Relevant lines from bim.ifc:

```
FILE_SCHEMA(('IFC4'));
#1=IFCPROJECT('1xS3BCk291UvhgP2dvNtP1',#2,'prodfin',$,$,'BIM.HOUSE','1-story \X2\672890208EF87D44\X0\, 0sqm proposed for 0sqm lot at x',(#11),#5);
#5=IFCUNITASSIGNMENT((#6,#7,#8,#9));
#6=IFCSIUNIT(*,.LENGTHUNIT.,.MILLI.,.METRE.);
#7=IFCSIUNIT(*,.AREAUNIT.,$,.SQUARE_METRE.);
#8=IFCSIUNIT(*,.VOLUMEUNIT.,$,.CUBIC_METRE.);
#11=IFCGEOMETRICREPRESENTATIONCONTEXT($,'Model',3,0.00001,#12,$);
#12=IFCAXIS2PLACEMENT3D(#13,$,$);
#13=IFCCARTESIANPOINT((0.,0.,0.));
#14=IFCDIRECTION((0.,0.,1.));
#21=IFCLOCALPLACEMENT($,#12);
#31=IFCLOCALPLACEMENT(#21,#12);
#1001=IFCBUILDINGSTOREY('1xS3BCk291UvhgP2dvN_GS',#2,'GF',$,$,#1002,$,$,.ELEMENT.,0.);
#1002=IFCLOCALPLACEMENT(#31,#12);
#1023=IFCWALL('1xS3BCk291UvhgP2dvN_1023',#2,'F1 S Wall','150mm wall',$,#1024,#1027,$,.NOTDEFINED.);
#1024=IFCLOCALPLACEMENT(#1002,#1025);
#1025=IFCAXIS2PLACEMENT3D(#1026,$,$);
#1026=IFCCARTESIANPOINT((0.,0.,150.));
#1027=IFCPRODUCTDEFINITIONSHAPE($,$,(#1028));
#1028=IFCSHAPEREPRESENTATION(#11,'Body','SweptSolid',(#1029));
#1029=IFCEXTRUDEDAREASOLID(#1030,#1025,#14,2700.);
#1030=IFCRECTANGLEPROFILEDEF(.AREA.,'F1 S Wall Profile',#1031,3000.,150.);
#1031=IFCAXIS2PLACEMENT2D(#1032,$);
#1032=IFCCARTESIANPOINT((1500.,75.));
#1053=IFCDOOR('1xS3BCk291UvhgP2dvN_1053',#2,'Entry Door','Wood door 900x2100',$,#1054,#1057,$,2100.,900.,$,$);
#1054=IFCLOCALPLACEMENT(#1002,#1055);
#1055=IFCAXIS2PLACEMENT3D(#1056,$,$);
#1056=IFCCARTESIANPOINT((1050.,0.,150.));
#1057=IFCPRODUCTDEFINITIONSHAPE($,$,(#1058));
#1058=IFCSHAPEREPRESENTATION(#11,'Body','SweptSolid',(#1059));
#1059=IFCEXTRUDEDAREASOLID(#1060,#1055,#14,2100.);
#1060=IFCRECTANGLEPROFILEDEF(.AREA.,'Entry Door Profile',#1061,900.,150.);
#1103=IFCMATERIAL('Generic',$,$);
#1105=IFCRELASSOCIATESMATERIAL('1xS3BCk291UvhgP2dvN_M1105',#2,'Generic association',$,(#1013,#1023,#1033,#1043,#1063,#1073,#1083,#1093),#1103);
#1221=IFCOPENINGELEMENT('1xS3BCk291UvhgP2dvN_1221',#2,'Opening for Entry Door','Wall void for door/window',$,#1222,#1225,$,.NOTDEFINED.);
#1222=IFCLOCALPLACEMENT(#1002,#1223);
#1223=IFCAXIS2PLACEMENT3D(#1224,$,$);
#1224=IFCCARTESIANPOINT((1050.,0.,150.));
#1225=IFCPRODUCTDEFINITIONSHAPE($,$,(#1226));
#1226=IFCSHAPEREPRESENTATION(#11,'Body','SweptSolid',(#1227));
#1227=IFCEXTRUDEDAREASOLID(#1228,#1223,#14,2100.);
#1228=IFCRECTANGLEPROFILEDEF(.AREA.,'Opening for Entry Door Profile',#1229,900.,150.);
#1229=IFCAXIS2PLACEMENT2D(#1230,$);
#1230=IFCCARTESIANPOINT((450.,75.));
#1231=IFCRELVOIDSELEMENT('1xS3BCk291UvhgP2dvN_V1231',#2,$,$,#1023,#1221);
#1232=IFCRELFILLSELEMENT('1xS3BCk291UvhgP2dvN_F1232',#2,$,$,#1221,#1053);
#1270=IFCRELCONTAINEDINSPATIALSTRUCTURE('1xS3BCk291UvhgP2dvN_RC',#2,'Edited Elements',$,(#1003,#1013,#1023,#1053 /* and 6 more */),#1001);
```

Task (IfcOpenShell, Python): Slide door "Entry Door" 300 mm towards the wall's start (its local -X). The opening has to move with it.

```python
import ifcopenshell
import ifcopenshell.api.geometry
import ifcopenshell.util.placement

model = ifcopenshell.open("bim.ifc")

door = model.by_guid("1xS3BCk291UvhgP2dvN_1053")
opening = door.FillsVoids[0].RelatingOpeningElement
wall = opening.VoidsElements[0].RelatingBuildingElement

wall_matrix = ifcopenshell.util.placement.get_local_placement(wall.ObjectPlacement)
shift = wall_matrix[:3, 0] * -300.0
before = ifcopenshell.util.placement.get_local_placement(door.ObjectPlacement)[:3, 3].copy()

# The door is not placed relative to its opening, so move both.
for product in (opening, door):
    matrix = ifcopenshell.util.placement.get_local_placement(product.ObjectPlacement)
    matrix[:3, 3] += shift
    ifcopenshell.api.geometry.edit_object_placement(model, product=product, matrix=matrix, is_si=False)

after = ifcopenshell.util.placement.get_local_placement(door.ObjectPlacement)[:3, 3]
print("door moved by", (after - before).round(3) + 0.0)

model.write("bim_updated.ifc")
```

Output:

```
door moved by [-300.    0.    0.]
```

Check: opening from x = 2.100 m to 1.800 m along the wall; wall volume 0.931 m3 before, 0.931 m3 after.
